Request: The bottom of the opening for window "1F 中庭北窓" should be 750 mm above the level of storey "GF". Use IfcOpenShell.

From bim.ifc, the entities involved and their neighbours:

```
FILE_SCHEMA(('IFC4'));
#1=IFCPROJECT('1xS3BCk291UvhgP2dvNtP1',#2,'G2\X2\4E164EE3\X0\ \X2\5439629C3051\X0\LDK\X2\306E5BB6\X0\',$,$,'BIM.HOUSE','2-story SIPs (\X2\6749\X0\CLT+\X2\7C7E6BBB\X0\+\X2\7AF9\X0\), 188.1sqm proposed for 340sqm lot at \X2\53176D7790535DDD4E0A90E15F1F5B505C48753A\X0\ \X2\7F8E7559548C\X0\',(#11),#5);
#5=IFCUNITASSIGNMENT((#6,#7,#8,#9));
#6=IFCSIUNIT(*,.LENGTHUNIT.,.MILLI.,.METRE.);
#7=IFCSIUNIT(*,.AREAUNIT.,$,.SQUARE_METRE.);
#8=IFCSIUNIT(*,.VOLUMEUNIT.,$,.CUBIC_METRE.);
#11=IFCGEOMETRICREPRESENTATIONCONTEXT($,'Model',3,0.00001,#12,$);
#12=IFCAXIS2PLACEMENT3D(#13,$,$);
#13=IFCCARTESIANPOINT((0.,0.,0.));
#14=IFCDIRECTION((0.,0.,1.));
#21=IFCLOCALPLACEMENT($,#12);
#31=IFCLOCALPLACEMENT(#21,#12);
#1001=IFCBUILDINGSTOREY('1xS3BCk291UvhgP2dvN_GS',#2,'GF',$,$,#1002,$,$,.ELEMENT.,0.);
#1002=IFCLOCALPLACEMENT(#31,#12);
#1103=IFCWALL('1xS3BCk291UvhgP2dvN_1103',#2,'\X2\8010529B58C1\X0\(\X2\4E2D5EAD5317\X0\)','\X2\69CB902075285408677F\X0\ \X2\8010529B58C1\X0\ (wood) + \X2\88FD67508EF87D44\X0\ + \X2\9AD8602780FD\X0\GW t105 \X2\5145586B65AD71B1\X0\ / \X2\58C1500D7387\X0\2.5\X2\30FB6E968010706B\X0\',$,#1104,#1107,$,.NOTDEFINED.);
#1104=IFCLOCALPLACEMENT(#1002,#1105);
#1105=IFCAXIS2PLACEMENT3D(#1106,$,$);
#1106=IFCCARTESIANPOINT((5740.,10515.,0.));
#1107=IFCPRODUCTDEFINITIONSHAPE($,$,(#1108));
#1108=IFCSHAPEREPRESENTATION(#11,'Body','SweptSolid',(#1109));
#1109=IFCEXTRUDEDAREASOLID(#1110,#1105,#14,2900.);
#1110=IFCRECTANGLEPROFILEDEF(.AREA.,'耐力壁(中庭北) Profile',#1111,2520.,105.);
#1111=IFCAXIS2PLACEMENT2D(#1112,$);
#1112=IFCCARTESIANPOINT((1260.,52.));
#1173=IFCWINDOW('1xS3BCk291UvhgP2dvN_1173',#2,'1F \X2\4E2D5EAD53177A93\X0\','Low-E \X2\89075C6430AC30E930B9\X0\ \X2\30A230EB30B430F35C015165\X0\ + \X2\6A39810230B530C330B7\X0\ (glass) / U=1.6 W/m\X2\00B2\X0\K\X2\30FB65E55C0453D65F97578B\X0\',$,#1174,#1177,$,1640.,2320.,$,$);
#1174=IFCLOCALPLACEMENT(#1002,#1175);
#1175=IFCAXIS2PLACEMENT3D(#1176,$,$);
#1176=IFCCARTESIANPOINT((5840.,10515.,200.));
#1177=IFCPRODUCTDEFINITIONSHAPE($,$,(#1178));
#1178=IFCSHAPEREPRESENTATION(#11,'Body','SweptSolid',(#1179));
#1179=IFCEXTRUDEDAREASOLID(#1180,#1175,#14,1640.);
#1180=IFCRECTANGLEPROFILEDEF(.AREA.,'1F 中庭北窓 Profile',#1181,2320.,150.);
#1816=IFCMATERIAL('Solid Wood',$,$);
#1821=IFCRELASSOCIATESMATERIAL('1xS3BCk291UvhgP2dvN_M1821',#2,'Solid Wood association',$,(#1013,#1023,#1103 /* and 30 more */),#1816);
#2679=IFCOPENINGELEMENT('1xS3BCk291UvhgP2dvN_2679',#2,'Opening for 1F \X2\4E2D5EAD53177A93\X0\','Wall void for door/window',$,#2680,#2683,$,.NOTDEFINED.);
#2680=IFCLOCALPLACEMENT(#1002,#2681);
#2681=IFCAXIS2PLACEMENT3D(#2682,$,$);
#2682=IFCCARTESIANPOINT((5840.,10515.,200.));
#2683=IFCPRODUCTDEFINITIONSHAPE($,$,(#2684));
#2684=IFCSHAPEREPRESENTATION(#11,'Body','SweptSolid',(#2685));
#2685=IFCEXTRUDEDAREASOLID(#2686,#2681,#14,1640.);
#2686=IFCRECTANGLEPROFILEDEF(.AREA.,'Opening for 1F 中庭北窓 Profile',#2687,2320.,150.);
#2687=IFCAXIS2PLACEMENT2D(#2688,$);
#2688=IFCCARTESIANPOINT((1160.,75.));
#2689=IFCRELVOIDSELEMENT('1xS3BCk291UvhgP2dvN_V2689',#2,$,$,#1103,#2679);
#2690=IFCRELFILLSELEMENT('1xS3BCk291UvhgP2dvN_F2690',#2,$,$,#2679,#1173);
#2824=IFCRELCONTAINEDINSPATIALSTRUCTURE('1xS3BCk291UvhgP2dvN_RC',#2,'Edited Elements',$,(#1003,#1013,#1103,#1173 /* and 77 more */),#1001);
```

```python
import numpy as np
import ifcopenshell
import ifcopenshell.api.geometry
import ifcopenshell.geom
import ifcopenshell.util.element
import ifcopenshell.util.placement
import ifcopenshell.util.shape
import ifcopenshell.util.unit

model = ifcopenshell.open("bim.ifc")
unit_scale = ifcopenshell.util.unit.calculate_unit_scale(model)

window = model.by_guid("1xS3BCk291UvhgP2dvN_1173")
opening = window.FillsVoids[0].RelatingOpeningElement
storey = ifcopenshell.util.element.get_container(window, ifc_class="IfcBuildingStorey")
level = ifcopenshell.util.placement.get_local_placement(storey.ObjectPlacement)[2, 3]

# The opening's origin need not be at the sill, so measure its lowest point.
shape = ifcopenshell.geom.create_shape(ifcopenshell.geom.settings(), opening)
bottom = ifcopenshell.util.shape.get_shape_bottom_elevation(shape, shape.geometry) / unit_scale
dz = level + 750.0 - bottom

shift = np.array([0.0, 0.0, dz])
# The window is not placed relative to its opening, so move both.
for product in (opening, window):
    matrix = ifcopenshell.util.placement.get_local_placement(product.ObjectPlacement)
    matrix[:3, 3] += shift
    ifcopenshell.api.geometry.edit_object_placement(model, product=product, matrix=matrix, is_si=False)

print(f"moved by {dz * unit_scale:+.3f} m")

model.write("bim_edited.ifc")
```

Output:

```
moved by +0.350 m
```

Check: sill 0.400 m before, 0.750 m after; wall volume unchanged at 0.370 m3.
